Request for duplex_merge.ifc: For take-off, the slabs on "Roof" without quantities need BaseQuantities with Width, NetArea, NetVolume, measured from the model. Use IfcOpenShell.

First a look at what the model holds.

```python
import ifcopenshell
import ifcopenshell.util.element
import ifcopenshell.util.unit

model = ifcopenshell.open("duplex_merge.ifc")
print(model.schema)
for unit_type in ("LENGTHUNIT", "AREAUNIT", "VOLUMEUNIT"):
    print(unit_type, ifcopenshell.util.unit.calculate_unit_scale(model, unit_type))
storey = next(s for s in model.by_type("IfcBuildingStorey") if s.Name == "Roof")
slabs = [e for e in ifcopenshell.util.element.get_decomposition(storey) if e.is_a("IfcSlab")]
for e in sorted(slabs, key=lambda e: e.id()):
    print(e.id(), e.is_a(), e.Name, list(ifcopenshell.util.element.get_psets(e, qtos_only=True)), sep=" | ")
```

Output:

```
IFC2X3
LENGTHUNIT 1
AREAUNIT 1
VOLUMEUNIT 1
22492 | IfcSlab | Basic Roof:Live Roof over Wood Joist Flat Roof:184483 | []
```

```python
import ifcopenshell
import ifcopenshell.api.pset
import ifcopenshell.geom
import ifcopenshell.util.element
import ifcopenshell.util.shape
import ifcopenshell.util.unit

model = ifcopenshell.open("duplex_merge.ifc")
unit_scale = ifcopenshell.util.unit.calculate_unit_scale(model)
area_scale = ifcopenshell.util.unit.calculate_unit_scale(model, "AREAUNIT")
volume_scale = ifcopenshell.util.unit.calculate_unit_scale(model, "VOLUMEUNIT")
settings = ifcopenshell.geom.settings()

storey = next(s for s in model.by_type("IfcBuildingStorey") if s.Name == "Roof")
slabs = [e for e in ifcopenshell.util.element.get_decomposition(storey) if e.is_a("IfcSlab")]

for e in sorted(slabs, key=lambda e: e.id()):
    if ifcopenshell.util.element.get_psets(e, qtos_only=True, should_inherit=False):
        continue
    # Geometry comes back in metres, in the element's own axes.
    shape = ifcopenshell.geom.create_shape(settings, e)
    values = {
        "Width": ifcopenshell.util.shape.get_z(shape.geometry) / unit_scale,
        "NetArea": ifcopenshell.util.shape.get_footprint_area(shape.geometry) / area_scale,
        "NetVolume": ifcopenshell.util.shape.get_volume(shape.geometry) / volume_scale,
    }
    qto = ifcopenshell.api.pset.add_qto(model, product=e, name="BaseQuantities")
    ifcopenshell.api.pset.edit_qto(model, qto=qto, properties=values)
    print(e.id(), {k: round(v, 3) for k, v in values.items()})

model.write("duplex_merge_updated.ifc")
```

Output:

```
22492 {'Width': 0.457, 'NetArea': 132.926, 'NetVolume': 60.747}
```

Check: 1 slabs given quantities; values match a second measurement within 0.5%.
